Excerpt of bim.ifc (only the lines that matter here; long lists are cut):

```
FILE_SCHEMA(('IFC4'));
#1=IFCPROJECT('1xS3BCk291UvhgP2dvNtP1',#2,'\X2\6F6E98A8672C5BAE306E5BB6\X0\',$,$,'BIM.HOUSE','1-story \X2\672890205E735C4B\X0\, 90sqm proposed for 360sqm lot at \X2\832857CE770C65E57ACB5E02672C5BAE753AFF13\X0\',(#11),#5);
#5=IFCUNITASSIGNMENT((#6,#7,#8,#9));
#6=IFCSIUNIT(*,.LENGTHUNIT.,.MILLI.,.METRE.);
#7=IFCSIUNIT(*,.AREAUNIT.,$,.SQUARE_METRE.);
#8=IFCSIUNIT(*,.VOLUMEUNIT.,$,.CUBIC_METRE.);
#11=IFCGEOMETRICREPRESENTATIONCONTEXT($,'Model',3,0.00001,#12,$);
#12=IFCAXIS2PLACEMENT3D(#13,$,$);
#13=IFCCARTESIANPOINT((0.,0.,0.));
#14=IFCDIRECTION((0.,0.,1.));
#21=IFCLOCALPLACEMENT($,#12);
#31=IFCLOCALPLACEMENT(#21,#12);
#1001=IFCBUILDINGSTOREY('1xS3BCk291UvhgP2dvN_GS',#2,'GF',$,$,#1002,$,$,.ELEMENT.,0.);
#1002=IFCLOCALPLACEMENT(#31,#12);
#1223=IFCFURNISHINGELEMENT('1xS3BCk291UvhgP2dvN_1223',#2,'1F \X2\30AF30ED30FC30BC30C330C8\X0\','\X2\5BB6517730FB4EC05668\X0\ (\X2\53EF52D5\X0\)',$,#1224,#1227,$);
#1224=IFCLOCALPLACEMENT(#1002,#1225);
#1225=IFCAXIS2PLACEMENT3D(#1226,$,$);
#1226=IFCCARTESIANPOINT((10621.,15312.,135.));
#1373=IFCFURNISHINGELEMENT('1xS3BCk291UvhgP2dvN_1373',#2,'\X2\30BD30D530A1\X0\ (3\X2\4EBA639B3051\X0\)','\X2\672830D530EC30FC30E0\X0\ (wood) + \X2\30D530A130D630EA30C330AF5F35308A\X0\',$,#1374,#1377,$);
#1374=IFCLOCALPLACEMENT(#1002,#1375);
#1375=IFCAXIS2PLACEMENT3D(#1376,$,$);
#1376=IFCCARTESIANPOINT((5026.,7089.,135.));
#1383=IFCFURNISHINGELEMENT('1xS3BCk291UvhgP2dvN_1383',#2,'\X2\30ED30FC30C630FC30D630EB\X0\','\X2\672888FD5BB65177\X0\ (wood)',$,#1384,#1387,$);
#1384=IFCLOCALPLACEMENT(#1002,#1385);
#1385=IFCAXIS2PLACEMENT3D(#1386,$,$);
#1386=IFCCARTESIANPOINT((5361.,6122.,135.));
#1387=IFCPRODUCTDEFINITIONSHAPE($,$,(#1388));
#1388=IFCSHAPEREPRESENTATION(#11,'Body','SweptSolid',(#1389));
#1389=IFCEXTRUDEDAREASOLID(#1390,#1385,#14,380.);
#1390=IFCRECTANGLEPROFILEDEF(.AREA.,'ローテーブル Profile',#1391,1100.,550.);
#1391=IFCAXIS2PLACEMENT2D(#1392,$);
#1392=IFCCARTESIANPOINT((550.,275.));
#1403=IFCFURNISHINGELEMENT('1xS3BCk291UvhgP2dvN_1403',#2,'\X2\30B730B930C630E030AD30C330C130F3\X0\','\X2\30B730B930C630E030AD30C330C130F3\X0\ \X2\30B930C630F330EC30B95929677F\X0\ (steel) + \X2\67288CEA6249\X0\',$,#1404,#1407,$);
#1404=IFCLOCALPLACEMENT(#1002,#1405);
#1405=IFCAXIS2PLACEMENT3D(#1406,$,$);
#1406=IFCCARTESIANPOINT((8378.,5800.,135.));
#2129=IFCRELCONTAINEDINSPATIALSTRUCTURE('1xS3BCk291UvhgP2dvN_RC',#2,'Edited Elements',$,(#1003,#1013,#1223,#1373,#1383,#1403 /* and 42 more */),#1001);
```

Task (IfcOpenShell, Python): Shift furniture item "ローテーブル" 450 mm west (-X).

```python
import ifcopenshell
import ifcopenshell.api.geometry
import ifcopenshell.util.placement
import ifcopenshell.util.unit

model = ifcopenshell.open("bim.ifc")
unit_scale = ifcopenshell.util.unit.calculate_unit_scale(model)

item = model.by_guid("1xS3BCk291UvhgP2dvN_1383")
matrix = ifcopenshell.util.placement.get_local_placement(item.ObjectPlacement)
matrix[0, 3] -= 0.45 / unit_scale
ifcopenshell.api.geometry.edit_object_placement(model, product=item, matrix=matrix, is_si=False)

print(ifcopenshell.util.placement.get_local_placement(item.ObjectPlacement).round(3) + 0.0)

model.write("bim-out.ifc")
```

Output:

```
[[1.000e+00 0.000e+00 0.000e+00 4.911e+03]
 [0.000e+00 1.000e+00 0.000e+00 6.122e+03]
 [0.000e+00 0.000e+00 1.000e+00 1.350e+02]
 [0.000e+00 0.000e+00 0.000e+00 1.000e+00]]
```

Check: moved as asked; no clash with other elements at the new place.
